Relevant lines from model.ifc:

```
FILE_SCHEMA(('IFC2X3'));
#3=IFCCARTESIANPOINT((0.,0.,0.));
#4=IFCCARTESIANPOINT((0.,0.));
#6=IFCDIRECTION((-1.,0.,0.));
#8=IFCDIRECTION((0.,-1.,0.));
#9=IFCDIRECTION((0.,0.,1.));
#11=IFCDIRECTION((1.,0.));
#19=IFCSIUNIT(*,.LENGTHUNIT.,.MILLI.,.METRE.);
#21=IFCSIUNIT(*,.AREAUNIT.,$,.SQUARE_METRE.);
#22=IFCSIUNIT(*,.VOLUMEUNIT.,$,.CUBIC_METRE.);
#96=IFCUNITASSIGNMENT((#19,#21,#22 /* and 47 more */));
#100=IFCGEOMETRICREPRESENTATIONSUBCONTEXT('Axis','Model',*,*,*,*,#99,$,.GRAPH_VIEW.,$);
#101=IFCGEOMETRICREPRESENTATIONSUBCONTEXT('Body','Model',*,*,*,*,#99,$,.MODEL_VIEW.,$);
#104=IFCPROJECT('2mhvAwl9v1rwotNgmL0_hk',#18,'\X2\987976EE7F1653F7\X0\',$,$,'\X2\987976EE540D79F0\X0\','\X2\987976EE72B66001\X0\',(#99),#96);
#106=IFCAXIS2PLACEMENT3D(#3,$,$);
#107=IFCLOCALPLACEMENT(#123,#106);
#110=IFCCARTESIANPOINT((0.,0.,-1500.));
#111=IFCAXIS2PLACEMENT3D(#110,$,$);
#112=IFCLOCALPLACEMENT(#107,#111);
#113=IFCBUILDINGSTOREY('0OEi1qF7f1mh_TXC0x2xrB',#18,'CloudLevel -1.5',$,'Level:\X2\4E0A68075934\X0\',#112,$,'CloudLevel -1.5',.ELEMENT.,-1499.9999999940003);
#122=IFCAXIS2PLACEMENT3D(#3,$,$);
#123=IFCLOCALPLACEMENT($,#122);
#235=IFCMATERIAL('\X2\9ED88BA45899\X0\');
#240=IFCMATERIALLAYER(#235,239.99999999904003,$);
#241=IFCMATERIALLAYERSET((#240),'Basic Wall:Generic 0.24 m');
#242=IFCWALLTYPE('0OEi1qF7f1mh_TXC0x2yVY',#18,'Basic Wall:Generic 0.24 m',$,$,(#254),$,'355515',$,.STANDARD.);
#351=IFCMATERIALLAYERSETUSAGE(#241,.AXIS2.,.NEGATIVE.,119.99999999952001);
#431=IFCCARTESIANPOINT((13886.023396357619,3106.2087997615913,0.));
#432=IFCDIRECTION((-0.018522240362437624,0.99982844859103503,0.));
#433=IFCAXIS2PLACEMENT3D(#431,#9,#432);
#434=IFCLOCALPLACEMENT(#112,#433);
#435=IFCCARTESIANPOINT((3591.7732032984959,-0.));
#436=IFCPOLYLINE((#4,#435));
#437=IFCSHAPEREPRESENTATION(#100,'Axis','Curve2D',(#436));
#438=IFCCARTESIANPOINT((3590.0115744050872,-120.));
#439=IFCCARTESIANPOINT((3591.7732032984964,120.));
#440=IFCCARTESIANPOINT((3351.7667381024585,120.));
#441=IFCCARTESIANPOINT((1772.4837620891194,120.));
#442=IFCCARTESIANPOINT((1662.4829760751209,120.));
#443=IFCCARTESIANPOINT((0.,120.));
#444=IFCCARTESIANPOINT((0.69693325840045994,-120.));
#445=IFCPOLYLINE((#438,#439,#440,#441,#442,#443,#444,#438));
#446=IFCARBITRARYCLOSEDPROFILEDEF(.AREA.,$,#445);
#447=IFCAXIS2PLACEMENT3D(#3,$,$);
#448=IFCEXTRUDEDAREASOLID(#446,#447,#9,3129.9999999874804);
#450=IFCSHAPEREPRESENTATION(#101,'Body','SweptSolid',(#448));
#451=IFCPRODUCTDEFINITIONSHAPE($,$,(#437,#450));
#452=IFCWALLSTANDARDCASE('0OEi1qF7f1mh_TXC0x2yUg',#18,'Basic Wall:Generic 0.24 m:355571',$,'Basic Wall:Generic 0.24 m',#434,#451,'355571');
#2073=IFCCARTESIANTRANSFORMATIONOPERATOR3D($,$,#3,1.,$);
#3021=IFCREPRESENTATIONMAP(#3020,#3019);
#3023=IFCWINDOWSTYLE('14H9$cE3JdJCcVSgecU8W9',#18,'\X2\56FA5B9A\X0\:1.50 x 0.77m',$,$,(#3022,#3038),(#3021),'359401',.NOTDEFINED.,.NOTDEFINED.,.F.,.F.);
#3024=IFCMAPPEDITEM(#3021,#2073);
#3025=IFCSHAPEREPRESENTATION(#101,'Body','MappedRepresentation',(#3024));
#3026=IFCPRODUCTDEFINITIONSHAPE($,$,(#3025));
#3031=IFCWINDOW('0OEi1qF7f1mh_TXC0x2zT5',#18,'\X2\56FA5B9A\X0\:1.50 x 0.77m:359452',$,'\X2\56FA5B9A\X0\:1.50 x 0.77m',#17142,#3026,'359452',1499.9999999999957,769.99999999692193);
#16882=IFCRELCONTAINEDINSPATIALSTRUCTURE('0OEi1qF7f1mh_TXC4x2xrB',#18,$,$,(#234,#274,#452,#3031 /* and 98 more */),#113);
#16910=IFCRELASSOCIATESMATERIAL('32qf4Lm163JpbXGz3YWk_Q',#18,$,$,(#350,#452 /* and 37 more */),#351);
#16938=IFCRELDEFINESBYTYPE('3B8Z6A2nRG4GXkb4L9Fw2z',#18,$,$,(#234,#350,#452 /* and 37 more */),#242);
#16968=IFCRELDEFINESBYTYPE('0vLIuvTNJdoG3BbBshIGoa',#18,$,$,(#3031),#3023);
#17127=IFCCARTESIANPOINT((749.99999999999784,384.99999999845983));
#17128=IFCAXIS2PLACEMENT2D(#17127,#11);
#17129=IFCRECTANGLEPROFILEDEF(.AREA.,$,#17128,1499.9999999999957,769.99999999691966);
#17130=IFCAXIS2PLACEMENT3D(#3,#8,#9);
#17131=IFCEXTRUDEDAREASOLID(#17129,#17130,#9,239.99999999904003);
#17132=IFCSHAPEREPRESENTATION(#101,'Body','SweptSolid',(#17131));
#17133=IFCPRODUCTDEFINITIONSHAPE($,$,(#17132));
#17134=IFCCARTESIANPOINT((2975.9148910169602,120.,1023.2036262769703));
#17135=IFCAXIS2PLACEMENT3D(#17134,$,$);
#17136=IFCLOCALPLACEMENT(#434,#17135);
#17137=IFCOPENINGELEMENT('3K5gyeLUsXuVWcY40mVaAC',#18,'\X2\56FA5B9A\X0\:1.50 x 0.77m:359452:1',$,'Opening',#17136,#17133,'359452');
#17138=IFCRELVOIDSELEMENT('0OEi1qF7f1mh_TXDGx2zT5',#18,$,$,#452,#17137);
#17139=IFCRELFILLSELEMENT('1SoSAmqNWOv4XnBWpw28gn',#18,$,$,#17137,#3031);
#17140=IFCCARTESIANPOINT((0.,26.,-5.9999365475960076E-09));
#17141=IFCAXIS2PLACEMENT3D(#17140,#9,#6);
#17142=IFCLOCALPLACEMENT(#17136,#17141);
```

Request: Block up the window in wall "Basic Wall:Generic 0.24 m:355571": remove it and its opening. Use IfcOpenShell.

```python
import ifcopenshell
import ifcopenshell.api.feature
import ifcopenshell.api.root
import ifcopenshell.geom
import ifcopenshell.util.shape

model = ifcopenshell.open("model.ifc")
settings = ifcopenshell.geom.settings()


def volume(element):
    """Net volume in cubic metres, openings subtracted."""
    shape = ifcopenshell.geom.create_shape(settings, element)
    return ifcopenshell.util.shape.get_volume(shape.geometry)


window = model.by_guid("0OEi1qF7f1mh_TXC0x2zT5")
opening = window.FillsVoids[0].RelatingOpeningElement
wall = opening.VoidsElements[0].RelatingBuildingElement
before = volume(wall)

ifcopenshell.api.root.remove_product(model, product=window)
ifcopenshell.api.feature.remove_feature(model, feature=opening)

after = volume(wall)

print(f"wall volume {before:.3f} -> {after:.3f} m3")

model.write("model_v2.ifc")
```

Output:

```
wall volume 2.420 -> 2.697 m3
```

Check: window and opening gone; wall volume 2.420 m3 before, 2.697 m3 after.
